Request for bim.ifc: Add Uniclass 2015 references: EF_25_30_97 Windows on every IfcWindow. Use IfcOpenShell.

First a look at what the model holds.

```python
import ifcopenshell

model = ifcopenshell.open("bim.ifc")
print(model.schema)
print("classifications:", [c.Name for c in model.by_type("IfcClassification")])
for ifc_class in ("IfcDoor", "IfcRoof", "IfcStair", "IfcWall", "IfcWindow"):
    print(ifc_class, len(model.by_type(ifc_class)))
```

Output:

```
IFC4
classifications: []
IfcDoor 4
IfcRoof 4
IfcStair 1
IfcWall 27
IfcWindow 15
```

```python
import ifcopenshell
import ifcopenshell.api.classification

model = ifcopenshell.open("bim.ifc")

system = ifcopenshell.api.classification.add_classification(model, classification="Uniclass 2015")

codes = {
    "IfcWindow": ("EF_25_30_97", "Windows"),
}
for ifc_class, (code, name) in codes.items():
    products = model.by_type(ifc_class)
    ifcopenshell.api.classification.add_reference(
        model, products=products, classification=system, identification=code, name=name
    )
    print(code, len(products))

model.write("bim_rev.ifc")
```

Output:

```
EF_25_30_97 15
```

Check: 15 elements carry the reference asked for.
